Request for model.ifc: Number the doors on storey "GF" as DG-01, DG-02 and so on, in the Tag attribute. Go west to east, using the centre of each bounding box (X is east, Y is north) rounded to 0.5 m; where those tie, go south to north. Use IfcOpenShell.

First a look at what the model holds.

```python
import ifcopenshell
import ifcopenshell.util.element
import ifcopenshell.util.placement

model = ifcopenshell.open("model.ifc")
print(model.schema)
storey = next(s for s in model.by_type("IfcBuildingStorey") if s.Name == "GF")
doors = [e for e in ifcopenshell.util.element.get_decomposition(storey) if e.is_a("IfcDoor")]
for e in sorted(doors, key=lambda e: e.id()):
    origin = ifcopenshell.util.placement.get_local_placement(e.ObjectPlacement)[:3, 3]
    print(e.id(), e.Tag, e.Name, origin.round(2) + 0.0, sep=" | ")
```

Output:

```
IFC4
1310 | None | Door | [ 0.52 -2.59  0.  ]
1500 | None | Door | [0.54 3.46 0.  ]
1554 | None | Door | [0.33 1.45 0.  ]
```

```python
import ifcopenshell
import ifcopenshell.geom
import ifcopenshell.util.element
import ifcopenshell.util.shape

model = ifcopenshell.open("model.ifc")
settings = ifcopenshell.geom.settings()
settings.set("use-world-coords", True)


def centre(element):
    shape = ifcopenshell.geom.create_shape(settings, element)
    return ifcopenshell.util.shape.get_bbox_centroid(shape.geometry)


storey = next(s for s in model.by_type("IfcBuildingStorey") if s.Name == "GF")
doors = [e for e in ifcopenshell.util.element.get_decomposition(storey) if e.is_a("IfcDoor")]

# Insertion points can sit at a corner or the storey origin, so sort by the geometry (in metres).
centres = {e: centre(e) for e in doors}
doors.sort(key=lambda e: (round(centres[e][0] / 0.5), centres[e][1]))

for i, e in enumerate(doors, start=1):
    number = f"DG-{i:02d}"
    e.Tag = number
    print(e.id(), number)

model.write("model_updated.ifc")
```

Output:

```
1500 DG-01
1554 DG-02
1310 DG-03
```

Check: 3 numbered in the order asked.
